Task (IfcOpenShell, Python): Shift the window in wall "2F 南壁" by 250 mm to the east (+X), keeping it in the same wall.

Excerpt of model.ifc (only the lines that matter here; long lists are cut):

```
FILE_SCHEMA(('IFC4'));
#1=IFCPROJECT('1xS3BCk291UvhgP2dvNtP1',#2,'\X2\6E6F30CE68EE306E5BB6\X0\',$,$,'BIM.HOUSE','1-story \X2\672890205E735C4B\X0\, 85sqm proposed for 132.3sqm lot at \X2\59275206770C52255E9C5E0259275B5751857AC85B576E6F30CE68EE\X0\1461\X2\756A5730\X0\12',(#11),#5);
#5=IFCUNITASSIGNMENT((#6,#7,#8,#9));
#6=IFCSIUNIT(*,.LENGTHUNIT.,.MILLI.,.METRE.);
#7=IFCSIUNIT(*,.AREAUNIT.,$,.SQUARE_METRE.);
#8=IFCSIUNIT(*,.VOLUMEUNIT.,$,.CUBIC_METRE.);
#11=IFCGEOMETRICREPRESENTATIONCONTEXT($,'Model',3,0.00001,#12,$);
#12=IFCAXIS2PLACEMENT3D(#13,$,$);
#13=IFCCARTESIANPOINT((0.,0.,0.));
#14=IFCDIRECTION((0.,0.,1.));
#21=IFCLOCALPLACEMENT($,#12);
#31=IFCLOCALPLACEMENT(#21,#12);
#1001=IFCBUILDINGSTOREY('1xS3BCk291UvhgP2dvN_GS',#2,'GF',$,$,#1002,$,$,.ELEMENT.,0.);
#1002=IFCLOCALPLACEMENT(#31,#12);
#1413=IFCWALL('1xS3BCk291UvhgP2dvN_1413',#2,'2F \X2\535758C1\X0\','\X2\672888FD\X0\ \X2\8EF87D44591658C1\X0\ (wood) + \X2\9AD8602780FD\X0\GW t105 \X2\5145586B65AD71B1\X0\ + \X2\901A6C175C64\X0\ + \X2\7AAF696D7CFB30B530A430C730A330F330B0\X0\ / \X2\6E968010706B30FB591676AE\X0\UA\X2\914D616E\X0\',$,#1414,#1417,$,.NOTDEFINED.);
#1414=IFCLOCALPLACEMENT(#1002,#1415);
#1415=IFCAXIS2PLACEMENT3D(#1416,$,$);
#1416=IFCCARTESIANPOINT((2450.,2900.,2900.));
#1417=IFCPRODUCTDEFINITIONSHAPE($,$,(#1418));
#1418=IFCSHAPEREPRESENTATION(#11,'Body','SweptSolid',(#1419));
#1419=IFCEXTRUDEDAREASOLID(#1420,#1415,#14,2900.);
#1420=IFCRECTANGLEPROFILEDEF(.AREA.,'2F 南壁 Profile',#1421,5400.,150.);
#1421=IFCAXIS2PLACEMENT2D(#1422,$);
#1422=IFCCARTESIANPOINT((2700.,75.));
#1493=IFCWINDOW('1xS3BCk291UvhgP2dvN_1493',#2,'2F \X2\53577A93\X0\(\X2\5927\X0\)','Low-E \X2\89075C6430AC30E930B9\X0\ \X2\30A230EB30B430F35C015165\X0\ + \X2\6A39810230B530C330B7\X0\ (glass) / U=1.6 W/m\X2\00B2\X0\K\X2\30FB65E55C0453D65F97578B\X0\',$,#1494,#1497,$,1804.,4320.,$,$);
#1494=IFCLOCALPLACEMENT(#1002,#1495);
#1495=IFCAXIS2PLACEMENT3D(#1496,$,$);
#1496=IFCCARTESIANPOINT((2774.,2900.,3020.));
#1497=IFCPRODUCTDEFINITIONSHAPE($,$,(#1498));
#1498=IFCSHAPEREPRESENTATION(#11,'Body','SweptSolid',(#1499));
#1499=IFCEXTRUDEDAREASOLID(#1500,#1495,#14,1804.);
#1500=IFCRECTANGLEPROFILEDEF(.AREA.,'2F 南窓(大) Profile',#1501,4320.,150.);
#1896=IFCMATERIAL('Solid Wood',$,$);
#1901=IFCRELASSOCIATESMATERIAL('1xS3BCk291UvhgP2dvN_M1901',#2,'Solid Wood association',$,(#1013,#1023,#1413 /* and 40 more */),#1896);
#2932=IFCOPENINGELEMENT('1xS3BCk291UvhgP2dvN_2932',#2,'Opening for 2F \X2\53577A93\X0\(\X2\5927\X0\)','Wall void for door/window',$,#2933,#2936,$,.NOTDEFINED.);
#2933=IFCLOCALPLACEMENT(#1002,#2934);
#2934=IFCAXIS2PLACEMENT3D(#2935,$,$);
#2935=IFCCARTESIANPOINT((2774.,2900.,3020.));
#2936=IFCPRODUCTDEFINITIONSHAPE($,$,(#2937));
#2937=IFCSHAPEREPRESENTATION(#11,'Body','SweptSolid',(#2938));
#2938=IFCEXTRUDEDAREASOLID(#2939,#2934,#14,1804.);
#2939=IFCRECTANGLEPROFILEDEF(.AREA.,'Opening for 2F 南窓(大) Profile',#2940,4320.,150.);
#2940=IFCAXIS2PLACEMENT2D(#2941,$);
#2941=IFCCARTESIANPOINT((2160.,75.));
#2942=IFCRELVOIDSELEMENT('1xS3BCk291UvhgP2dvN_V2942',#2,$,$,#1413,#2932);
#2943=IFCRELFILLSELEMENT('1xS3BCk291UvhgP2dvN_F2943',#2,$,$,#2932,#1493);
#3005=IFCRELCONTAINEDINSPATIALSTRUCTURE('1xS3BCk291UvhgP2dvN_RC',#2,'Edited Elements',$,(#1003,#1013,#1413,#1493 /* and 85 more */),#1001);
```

```python
import ifcopenshell
import ifcopenshell.api.geometry
import ifcopenshell.util.placement
import ifcopenshell.util.unit

model = ifcopenshell.open("model.ifc")
unit_scale = ifcopenshell.util.unit.calculate_unit_scale(model)

window = model.by_id(1493)
opening = window.FillsVoids[0].RelatingOpeningElement
wall = opening.VoidsElements[0].RelatingBuildingElement

wall_matrix = ifcopenshell.util.placement.get_local_placement(wall.ObjectPlacement)
shift = wall_matrix[:3, 0] * 0.25 / unit_scale
before = ifcopenshell.util.placement.get_local_placement(window.ObjectPlacement)[:3, 3].copy()

# The window is not placed relative to its opening, so move both.
for product in (opening, window):
    matrix = ifcopenshell.util.placement.get_local_placement(product.ObjectPlacement)
    matrix[:3, 3] += shift
    ifcopenshell.api.geometry.edit_object_placement(model, product=product, matrix=matrix, is_si=False)

after = ifcopenshell.util.placement.get_local_placement(window.ObjectPlacement)[:3, 3]
print("window moved by", (after - before).round(3) + 0.0)

model.write("model_edited.ifc")
```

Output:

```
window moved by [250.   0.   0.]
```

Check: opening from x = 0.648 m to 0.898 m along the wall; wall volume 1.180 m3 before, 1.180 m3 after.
